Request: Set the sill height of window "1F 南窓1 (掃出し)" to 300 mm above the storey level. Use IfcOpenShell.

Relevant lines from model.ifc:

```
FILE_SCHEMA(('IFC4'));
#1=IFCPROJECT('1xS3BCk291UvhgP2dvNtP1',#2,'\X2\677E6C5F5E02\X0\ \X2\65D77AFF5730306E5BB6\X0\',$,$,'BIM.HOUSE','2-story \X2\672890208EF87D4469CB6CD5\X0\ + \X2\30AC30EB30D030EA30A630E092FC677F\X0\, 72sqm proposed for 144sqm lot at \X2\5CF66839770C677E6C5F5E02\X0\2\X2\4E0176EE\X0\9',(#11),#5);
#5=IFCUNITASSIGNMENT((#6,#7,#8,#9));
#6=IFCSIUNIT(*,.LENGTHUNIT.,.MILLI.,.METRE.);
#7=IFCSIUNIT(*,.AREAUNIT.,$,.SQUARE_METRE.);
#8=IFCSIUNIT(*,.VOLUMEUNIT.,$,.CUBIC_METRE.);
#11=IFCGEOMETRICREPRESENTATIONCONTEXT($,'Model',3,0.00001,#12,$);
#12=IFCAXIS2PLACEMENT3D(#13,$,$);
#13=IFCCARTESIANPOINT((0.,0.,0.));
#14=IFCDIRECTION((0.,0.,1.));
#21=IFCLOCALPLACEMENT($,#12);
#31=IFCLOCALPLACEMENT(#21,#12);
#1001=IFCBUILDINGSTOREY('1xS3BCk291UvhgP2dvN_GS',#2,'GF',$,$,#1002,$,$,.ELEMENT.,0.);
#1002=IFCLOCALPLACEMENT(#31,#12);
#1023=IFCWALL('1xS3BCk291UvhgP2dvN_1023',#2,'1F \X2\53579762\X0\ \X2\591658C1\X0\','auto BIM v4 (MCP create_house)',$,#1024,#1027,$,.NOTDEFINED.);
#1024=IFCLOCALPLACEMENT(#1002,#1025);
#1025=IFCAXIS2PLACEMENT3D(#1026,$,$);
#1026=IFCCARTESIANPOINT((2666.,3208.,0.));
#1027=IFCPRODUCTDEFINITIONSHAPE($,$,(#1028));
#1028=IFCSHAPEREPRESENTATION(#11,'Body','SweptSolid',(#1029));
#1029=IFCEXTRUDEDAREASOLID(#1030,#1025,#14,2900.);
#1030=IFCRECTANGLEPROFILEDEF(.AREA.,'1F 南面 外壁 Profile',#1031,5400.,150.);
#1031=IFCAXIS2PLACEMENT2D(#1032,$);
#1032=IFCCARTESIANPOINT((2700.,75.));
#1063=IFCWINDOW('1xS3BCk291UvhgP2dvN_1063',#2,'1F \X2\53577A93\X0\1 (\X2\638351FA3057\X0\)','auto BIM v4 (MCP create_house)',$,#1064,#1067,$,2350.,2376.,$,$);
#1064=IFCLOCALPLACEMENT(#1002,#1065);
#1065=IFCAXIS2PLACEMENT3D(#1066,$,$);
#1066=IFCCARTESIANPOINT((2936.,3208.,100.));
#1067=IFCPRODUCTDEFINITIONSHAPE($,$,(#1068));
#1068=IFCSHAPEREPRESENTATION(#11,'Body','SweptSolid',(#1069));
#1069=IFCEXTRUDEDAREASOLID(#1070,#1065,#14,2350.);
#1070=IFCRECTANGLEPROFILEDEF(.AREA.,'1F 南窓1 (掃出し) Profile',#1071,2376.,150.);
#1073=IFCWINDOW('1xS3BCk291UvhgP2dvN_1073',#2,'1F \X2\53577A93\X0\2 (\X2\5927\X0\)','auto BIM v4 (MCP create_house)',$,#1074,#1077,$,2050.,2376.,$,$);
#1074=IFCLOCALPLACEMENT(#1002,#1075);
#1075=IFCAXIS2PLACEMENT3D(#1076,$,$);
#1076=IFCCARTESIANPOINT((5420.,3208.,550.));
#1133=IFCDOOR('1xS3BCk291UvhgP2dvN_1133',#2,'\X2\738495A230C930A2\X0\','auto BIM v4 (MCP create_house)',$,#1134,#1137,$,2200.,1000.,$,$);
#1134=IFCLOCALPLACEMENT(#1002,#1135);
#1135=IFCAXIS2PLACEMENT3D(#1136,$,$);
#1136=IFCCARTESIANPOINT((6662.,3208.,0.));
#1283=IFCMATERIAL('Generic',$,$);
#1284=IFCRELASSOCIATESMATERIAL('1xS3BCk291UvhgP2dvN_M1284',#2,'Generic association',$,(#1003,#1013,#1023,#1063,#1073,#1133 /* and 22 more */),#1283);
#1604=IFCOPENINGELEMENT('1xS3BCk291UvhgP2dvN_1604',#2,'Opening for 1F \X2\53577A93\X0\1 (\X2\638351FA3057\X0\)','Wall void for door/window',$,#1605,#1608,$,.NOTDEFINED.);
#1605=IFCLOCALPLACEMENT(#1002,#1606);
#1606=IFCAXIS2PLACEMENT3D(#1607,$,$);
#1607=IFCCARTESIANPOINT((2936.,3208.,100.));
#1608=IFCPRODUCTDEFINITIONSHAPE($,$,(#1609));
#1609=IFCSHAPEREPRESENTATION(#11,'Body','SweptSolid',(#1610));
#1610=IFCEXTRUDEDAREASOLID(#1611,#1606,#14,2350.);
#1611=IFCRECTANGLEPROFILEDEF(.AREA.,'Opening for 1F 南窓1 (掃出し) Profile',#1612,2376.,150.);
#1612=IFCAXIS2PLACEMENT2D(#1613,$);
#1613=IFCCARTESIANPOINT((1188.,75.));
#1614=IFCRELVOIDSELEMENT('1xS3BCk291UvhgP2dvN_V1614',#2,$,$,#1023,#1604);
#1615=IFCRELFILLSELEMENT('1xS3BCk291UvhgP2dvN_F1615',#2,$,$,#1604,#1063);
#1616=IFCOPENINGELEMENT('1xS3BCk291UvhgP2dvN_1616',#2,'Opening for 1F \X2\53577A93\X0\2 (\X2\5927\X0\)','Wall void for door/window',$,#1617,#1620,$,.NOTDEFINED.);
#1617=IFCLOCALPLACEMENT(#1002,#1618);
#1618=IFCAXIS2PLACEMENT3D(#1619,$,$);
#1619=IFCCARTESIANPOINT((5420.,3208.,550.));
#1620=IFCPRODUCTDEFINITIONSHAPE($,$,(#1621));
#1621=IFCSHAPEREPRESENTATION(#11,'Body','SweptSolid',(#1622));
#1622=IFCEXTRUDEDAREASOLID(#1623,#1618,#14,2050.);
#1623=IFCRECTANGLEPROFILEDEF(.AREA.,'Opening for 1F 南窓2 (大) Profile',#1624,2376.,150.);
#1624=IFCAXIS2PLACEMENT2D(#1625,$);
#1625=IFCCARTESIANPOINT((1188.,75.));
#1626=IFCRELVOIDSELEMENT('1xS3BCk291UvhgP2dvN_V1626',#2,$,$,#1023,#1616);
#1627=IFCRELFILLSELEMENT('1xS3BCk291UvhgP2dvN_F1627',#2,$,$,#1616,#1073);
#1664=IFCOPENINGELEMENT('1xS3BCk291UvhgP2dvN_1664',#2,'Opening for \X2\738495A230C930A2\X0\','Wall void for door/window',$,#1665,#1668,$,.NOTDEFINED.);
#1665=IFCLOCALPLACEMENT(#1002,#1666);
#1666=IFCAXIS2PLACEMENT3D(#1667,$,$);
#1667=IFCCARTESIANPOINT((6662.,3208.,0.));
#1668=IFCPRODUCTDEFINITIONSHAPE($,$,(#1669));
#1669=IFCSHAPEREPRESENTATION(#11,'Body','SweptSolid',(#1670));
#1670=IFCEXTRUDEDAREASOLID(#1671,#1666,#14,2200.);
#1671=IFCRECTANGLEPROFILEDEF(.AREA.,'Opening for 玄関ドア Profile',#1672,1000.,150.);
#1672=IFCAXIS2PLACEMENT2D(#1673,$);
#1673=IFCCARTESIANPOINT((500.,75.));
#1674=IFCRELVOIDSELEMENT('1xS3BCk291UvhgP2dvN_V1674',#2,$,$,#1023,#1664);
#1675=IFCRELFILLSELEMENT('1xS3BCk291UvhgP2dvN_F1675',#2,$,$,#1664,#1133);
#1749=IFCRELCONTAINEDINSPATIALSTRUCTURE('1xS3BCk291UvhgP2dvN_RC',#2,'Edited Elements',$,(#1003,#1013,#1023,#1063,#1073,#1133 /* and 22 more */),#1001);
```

```python
import numpy as np
import ifcopenshell
import ifcopenshell.api.geometry
import ifcopenshell.geom
import ifcopenshell.util.element
import ifcopenshell.util.placement
import ifcopenshell.util.shape
import ifcopenshell.util.unit

model = ifcopenshell.open("model.ifc")
unit_scale = ifcopenshell.util.unit.calculate_unit_scale(model)

window = model.by_id(1063)
opening = window.FillsVoids[0].RelatingOpeningElement
storey = ifcopenshell.util.element.get_container(window, ifc_class="IfcBuildingStorey")
level = ifcopenshell.util.placement.get_local_placement(storey.ObjectPlacement)[2, 3]

# The opening's origin need not be at the sill, so measure its lowest point.
shape = ifcopenshell.geom.create_shape(ifcopenshell.geom.settings(), opening)
bottom = ifcopenshell.util.shape.get_shape_bottom_elevation(shape, shape.geometry) / unit_scale
dz = level + 0.3 / unit_scale - bottom

shift = np.array([0.0, 0.0, dz])
# The window is not placed relative to its opening, so move both.
for product in (opening, window):
    matrix = ifcopenshell.util.placement.get_local_placement(product.ObjectPlacement)
    matrix[:3, 3] += shift
    ifcopenshell.api.geometry.edit_object_placement(model, product=product, matrix=matrix, is_si=False)

print(f"moved by {dz * unit_scale:+.3f} m")

model.write("model_edited.ifc")
```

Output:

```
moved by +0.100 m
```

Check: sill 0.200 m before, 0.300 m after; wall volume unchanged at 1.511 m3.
